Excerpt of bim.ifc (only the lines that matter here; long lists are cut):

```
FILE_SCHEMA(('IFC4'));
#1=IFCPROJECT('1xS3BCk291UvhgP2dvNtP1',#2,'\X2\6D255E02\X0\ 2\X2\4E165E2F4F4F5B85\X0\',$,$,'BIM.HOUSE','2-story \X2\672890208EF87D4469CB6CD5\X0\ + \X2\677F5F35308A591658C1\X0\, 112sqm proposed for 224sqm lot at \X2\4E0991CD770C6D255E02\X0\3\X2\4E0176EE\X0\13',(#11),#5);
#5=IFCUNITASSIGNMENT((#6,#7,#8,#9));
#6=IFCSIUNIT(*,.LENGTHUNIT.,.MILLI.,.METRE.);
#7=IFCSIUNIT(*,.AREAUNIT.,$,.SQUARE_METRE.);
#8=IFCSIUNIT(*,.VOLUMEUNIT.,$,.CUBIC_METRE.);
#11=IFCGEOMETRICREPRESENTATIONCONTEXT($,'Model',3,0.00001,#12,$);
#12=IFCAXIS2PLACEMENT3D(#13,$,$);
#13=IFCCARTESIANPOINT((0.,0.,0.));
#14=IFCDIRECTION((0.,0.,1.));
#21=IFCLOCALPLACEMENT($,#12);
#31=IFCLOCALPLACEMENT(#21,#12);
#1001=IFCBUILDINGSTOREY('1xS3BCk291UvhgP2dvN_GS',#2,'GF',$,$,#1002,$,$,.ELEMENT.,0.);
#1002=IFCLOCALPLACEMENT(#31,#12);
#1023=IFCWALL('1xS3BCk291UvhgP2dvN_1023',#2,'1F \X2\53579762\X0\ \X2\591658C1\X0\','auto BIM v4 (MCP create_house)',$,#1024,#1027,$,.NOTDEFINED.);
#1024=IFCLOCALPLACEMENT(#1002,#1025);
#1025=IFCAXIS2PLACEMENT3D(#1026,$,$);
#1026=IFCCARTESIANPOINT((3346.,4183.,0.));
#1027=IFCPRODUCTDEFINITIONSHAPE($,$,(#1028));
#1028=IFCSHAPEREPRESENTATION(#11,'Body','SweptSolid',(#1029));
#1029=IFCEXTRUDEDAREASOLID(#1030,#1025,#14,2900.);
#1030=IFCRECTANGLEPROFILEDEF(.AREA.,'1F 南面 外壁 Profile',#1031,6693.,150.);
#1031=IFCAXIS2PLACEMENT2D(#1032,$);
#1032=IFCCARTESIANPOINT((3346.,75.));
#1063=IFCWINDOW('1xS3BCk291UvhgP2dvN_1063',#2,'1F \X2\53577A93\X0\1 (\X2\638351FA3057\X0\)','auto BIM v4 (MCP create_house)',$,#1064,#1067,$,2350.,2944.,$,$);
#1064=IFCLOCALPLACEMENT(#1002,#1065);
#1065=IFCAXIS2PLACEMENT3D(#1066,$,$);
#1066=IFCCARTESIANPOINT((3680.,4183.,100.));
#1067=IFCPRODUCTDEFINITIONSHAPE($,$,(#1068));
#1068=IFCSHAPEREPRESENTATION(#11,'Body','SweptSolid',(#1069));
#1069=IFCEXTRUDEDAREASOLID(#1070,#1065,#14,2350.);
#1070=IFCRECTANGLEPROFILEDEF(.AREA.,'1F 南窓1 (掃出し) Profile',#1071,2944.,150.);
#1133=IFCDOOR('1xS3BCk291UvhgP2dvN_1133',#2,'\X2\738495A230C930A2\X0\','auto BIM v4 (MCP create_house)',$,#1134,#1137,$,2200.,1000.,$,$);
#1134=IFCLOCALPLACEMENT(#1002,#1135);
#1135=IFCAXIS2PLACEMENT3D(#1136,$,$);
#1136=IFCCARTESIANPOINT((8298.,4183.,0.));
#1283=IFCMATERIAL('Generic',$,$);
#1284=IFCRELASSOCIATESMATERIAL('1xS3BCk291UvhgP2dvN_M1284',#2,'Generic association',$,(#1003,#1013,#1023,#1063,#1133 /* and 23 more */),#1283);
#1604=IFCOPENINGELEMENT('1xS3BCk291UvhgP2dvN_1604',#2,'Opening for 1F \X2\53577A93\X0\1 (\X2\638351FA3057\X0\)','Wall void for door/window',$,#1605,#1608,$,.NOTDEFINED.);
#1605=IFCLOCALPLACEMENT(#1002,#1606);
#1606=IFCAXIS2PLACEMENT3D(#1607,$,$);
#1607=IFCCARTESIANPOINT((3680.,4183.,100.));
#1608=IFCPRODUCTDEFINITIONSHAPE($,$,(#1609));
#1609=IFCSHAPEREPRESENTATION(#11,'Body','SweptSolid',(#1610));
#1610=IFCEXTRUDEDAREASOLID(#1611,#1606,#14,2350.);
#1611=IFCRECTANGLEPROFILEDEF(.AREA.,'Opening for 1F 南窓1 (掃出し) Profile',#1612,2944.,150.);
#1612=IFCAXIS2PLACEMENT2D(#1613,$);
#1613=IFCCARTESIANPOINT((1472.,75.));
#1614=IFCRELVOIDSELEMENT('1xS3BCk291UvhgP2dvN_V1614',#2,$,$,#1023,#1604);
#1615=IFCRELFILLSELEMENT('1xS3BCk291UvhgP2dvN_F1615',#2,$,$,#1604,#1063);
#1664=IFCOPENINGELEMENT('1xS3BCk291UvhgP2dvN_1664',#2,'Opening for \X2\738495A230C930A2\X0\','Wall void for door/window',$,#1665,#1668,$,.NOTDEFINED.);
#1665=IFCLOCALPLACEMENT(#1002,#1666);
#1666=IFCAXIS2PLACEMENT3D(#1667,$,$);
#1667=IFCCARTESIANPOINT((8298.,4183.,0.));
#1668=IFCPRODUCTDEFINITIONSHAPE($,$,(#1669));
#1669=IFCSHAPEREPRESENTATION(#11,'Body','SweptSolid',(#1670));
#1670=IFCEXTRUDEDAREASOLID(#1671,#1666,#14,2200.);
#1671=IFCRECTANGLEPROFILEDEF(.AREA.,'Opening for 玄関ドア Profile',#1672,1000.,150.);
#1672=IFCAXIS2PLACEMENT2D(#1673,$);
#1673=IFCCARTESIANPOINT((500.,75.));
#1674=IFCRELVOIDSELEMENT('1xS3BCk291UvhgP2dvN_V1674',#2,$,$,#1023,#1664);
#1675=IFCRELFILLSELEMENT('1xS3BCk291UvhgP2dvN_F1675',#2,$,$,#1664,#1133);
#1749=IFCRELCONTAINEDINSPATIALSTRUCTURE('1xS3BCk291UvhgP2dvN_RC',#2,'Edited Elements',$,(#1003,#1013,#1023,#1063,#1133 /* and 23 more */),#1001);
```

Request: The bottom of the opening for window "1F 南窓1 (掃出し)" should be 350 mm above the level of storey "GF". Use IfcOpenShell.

```python
import numpy as np
import ifcopenshell
import ifcopenshell.api.geometry
import ifcopenshell.geom
import ifcopenshell.util.element
import ifcopenshell.util.placement
import ifcopenshell.util.shape
import ifcopenshell.util.unit

model = ifcopenshell.open("bim.ifc")
unit_scale = ifcopenshell.util.unit.calculate_unit_scale(model)

window = model.by_guid("1xS3BCk291UvhgP2dvN_1063")
opening = window.FillsVoids[0].RelatingOpeningElement
storey = ifcopenshell.util.element.get_container(window, ifc_class="IfcBuildingStorey")
level = ifcopenshell.util.placement.get_local_placement(storey.ObjectPlacement)[2, 3]

# The opening's origin need not be at the sill, so measure its lowest point.
shape = ifcopenshell.geom.create_shape(ifcopenshell.geom.settings(), opening)
bottom = ifcopenshell.util.shape.get_shape_bottom_elevation(shape, shape.geometry) / unit_scale
dz = level + 0.35 / unit_scale - bottom

shift = np.array([0.0, 0.0, dz])
# The window is not placed relative to its opening, so move both.
for product in (opening, window):
    matrix = ifcopenshell.util.placement.get_local_placement(product.ObjectPlacement)
    matrix[:3, 3] += shift
    ifcopenshell.api.geometry.edit_object_placement(model, product=product, matrix=matrix, is_si=False)

print(f"moved by {dz * unit_scale:+.3f} m")

model.write("bim_v2.ifc")
```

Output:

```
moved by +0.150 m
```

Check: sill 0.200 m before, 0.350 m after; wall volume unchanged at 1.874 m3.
